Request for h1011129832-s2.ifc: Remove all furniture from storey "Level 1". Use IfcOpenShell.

First a look at what the model holds.

```python
import ifcopenshell
import ifcopenshell.util.element

model = ifcopenshell.open("h1011129832-s2.ifc")
print(model.schema)
storey = next(s for s in model.by_type("IfcBuildingStorey") if s.Name == "Level 1")
furniture = [e for e in ifcopenshell.util.element.get_decomposition(storey) if e.is_a("IfcFurnishingElement")]
seen = {}
for e in furniture:
    element_type = ifcopenshell.util.element.get_type(e)
    name = element_type.Name if element_type not in (None, e) else None
    seen[name] = seen.get(name, 0) + 1
for name, count in sorted(seen.items(), key=str):
    print(count, "x", name)
```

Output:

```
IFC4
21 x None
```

```python
import ifcopenshell
import ifcopenshell.api.root
import ifcopenshell.util.element

model = ifcopenshell.open("h1011129832-s2.ifc")

storey = next(s for s in model.by_type("IfcBuildingStorey") if s.Name == "Level 1")
furniture = [e for e in ifcopenshell.util.element.get_decomposition(storey) if e.is_a("IfcFurnishingElement")]

for e in furniture:
    ifcopenshell.api.root.remove_product(model, product=e)
print(len(furniture), "removed")

model.write("h1011129832-s2_updated.ifc")
```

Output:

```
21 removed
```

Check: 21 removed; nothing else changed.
